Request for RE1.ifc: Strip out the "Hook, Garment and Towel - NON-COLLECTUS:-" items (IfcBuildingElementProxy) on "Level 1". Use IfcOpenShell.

First a look at what the model holds.

```python
import ifcopenshell
import ifcopenshell.util.element

model = ifcopenshell.open("RE1.ifc")
print(model.schema)
storey = next(s for s in model.by_type("IfcBuildingStorey") if s.Name == "Level 1")
proxies = [e for e in ifcopenshell.util.element.get_decomposition(storey) if e.is_a("IfcBuildingElementProxy")]
seen = {}
for e in proxies:
    element_type = ifcopenshell.util.element.get_type(e)
    name = element_type.Name if element_type not in (None, e) else None
    seen[name] = seen.get(name, 0) + 1
for name, count in sorted(seen.items(), key=str):
    print(count, "x", name)
```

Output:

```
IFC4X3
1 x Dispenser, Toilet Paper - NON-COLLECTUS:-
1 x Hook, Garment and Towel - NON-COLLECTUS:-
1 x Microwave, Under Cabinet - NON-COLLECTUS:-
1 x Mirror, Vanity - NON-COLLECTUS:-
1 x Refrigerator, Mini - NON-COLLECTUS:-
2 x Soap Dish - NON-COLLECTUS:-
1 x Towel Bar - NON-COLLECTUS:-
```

```python
import ifcopenshell
import ifcopenshell.api.root
import ifcopenshell.util.element

model = ifcopenshell.open("RE1.ifc")

storey = next(s for s in model.by_type("IfcBuildingStorey") if s.Name == "Level 1")
proxies = [e for e in ifcopenshell.util.element.get_decomposition(storey) if e.is_a("IfcBuildingElementProxy")]
targets = [e for e in proxies if (t := ifcopenshell.util.element.get_type(e)) not in (None, e) and t.Name == "Hook, Garment and Towel - NON-COLLECTUS:-"]

for e in targets:
    ifcopenshell.api.root.remove_product(model, product=e)
print(len(targets), "removed")

model.write("RE1_v2.ifc")
```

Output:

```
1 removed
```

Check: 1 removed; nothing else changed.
